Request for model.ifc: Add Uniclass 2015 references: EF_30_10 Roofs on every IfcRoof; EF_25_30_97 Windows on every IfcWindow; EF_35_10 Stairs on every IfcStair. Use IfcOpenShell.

First a look at what the model holds.

```python
import ifcopenshell

model = ifcopenshell.open("model.ifc")
print(model.schema)
print("classifications:", [c.Name for c in model.by_type("IfcClassification")])
for ifc_class in ("IfcDoor", "IfcRoof", "IfcStair", "IfcWall", "IfcWindow"):
    print(ifc_class, len(model.by_type(ifc_class)))
```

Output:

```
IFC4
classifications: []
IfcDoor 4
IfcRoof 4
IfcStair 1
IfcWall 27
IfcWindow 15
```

```python
import ifcopenshell
import ifcopenshell.api.classification

model = ifcopenshell.open("model.ifc")

system = ifcopenshell.api.classification.add_classification(model, classification="Uniclass 2015")

codes = {
    "IfcRoof": ("EF_30_10", "Roofs"),
    "IfcWindow": ("EF_25_30_97", "Windows"),
    "IfcStair": ("EF_35_10", "Stairs"),
}
for ifc_class, (code, name) in codes.items():
    products = model.by_type(ifc_class)
    ifcopenshell.api.classification.add_reference(
        model, products=products, classification=system, identification=code, name=name
    )
    print(code, len(products))

model.write("model_edited.ifc")
```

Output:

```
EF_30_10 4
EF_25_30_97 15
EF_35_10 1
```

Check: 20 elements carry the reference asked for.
